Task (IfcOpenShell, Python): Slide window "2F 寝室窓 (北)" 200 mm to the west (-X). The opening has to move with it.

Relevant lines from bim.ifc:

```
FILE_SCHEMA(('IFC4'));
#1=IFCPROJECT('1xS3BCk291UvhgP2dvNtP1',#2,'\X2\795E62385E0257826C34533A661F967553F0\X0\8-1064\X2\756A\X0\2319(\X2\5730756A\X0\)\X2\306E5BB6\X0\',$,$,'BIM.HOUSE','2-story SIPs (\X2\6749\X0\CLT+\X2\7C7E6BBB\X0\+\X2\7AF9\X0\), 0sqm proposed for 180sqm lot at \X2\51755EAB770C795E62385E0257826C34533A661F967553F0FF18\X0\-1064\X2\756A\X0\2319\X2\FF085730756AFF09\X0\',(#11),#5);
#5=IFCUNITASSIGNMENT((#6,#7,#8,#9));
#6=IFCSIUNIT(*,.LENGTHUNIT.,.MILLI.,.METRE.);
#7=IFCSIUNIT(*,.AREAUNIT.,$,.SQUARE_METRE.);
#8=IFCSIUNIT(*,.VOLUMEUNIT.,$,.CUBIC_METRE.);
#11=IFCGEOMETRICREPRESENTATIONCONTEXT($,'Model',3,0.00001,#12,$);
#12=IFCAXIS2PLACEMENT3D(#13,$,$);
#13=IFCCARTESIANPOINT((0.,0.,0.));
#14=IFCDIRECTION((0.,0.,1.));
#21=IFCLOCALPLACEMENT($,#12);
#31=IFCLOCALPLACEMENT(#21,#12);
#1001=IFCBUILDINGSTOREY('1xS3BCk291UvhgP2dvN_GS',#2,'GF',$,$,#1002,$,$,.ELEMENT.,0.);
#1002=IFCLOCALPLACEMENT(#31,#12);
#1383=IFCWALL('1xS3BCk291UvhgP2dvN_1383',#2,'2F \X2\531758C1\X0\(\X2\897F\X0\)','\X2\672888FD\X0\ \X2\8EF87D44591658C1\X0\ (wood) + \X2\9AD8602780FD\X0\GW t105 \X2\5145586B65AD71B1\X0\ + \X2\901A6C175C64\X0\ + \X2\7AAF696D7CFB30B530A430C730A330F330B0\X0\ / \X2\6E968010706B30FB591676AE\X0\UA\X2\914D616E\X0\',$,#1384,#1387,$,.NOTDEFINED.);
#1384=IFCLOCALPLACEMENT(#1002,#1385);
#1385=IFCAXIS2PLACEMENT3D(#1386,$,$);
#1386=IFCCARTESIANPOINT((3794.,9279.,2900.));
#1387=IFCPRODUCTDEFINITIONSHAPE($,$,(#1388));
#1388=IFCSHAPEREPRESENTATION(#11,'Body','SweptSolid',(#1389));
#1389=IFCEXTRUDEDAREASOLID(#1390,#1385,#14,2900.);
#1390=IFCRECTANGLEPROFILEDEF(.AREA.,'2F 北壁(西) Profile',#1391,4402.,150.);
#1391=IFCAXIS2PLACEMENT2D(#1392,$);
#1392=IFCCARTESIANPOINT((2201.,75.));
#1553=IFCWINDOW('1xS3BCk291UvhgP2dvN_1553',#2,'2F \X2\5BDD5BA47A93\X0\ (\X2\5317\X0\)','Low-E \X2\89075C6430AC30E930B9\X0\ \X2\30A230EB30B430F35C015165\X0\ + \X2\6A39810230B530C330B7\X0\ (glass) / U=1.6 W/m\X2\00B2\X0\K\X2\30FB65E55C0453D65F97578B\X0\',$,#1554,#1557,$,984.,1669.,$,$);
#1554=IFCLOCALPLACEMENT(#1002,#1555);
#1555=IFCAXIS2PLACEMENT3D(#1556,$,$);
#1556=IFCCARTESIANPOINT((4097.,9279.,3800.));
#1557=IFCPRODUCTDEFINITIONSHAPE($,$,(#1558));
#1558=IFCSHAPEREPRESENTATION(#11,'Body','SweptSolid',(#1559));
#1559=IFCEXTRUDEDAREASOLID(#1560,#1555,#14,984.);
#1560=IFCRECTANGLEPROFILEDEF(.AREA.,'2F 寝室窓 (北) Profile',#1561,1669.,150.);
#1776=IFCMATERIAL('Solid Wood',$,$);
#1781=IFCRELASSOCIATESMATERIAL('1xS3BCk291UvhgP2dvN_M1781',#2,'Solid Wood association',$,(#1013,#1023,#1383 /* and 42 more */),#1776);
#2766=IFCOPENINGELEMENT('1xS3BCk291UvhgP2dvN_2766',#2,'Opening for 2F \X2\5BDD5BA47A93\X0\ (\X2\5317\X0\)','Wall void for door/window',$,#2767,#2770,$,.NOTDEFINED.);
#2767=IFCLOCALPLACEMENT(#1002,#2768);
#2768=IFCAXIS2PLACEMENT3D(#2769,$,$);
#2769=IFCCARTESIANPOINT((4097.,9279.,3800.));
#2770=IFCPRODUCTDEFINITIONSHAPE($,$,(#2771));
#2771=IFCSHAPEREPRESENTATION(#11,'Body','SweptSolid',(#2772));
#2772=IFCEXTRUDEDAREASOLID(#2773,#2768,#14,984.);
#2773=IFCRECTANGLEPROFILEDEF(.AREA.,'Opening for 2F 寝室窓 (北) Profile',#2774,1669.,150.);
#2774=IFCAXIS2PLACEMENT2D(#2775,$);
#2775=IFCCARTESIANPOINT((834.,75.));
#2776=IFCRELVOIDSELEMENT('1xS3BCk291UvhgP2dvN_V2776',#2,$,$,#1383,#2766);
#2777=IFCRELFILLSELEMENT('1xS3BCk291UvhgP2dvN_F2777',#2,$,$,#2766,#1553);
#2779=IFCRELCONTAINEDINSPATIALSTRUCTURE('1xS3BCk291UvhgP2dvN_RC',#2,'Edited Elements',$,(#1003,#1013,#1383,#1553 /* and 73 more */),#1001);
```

```python
import ifcopenshell
import ifcopenshell.api.geometry
import ifcopenshell.util.placement

model = ifcopenshell.open("bim.ifc")

window = model.by_guid("1xS3BCk291UvhgP2dvN_1553")
opening = window.FillsVoids[0].RelatingOpeningElement
wall = opening.VoidsElements[0].RelatingBuildingElement

wall_matrix = ifcopenshell.util.placement.get_local_placement(wall.ObjectPlacement)
shift = wall_matrix[:3, 0] * -200.0
before = ifcopenshell.util.placement.get_local_placement(window.ObjectPlacement)[:3, 3].copy()

# The window is not placed relative to its opening, so move both.
for product in (opening, window):
    matrix = ifcopenshell.util.placement.get_local_placement(product.ObjectPlacement)
    matrix[:3, 3] += shift
    ifcopenshell.api.geometry.edit_object_placement(model, product=product, matrix=matrix, is_si=False)

after = ifcopenshell.util.placement.get_local_placement(window.ObjectPlacement)[:3, 3]
print("window moved by", (after - before).round(3) + 0.0)

model.write("bim_rev.ifc")
```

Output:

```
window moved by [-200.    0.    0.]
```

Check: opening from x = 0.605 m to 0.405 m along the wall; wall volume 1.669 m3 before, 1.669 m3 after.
